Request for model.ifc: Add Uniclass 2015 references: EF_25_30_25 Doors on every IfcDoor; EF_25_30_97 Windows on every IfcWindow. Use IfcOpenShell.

First a look at what the model holds.

```python
import ifcopenshell

model = ifcopenshell.open("model.ifc")
print(model.schema)
print("classifications:", [c.Name for c in model.by_type("IfcClassification")])
for ifc_class in ("IfcDoor", "IfcRoof", "IfcStair", "IfcWall", "IfcWindow"):
    print(ifc_class, len(model.by_type(ifc_class)))
```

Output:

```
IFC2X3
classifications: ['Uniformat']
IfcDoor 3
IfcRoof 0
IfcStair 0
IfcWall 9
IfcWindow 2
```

```python
import ifcopenshell
import ifcopenshell.api.classification

model = ifcopenshell.open("model.ifc")

# IFC2X3 requires Source and Edition and has no link from the project to the system.
system = model.create_entity("IfcClassification", Source="NBS", Edition="2015", Name="Uniclass 2015")

codes = {
    "IfcDoor": ("EF_25_30_25", "Doors"),
    "IfcWindow": ("EF_25_30_97", "Windows"),
}
for ifc_class, (code, name) in codes.items():
    products = model.by_type(ifc_class)
    ifcopenshell.api.classification.add_reference(
        model, products=products, classification=system, identification=code, name=name
    )
    print(code, len(products))

model.write("model_v2.ifc")
```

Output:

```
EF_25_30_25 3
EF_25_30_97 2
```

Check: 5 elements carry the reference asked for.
